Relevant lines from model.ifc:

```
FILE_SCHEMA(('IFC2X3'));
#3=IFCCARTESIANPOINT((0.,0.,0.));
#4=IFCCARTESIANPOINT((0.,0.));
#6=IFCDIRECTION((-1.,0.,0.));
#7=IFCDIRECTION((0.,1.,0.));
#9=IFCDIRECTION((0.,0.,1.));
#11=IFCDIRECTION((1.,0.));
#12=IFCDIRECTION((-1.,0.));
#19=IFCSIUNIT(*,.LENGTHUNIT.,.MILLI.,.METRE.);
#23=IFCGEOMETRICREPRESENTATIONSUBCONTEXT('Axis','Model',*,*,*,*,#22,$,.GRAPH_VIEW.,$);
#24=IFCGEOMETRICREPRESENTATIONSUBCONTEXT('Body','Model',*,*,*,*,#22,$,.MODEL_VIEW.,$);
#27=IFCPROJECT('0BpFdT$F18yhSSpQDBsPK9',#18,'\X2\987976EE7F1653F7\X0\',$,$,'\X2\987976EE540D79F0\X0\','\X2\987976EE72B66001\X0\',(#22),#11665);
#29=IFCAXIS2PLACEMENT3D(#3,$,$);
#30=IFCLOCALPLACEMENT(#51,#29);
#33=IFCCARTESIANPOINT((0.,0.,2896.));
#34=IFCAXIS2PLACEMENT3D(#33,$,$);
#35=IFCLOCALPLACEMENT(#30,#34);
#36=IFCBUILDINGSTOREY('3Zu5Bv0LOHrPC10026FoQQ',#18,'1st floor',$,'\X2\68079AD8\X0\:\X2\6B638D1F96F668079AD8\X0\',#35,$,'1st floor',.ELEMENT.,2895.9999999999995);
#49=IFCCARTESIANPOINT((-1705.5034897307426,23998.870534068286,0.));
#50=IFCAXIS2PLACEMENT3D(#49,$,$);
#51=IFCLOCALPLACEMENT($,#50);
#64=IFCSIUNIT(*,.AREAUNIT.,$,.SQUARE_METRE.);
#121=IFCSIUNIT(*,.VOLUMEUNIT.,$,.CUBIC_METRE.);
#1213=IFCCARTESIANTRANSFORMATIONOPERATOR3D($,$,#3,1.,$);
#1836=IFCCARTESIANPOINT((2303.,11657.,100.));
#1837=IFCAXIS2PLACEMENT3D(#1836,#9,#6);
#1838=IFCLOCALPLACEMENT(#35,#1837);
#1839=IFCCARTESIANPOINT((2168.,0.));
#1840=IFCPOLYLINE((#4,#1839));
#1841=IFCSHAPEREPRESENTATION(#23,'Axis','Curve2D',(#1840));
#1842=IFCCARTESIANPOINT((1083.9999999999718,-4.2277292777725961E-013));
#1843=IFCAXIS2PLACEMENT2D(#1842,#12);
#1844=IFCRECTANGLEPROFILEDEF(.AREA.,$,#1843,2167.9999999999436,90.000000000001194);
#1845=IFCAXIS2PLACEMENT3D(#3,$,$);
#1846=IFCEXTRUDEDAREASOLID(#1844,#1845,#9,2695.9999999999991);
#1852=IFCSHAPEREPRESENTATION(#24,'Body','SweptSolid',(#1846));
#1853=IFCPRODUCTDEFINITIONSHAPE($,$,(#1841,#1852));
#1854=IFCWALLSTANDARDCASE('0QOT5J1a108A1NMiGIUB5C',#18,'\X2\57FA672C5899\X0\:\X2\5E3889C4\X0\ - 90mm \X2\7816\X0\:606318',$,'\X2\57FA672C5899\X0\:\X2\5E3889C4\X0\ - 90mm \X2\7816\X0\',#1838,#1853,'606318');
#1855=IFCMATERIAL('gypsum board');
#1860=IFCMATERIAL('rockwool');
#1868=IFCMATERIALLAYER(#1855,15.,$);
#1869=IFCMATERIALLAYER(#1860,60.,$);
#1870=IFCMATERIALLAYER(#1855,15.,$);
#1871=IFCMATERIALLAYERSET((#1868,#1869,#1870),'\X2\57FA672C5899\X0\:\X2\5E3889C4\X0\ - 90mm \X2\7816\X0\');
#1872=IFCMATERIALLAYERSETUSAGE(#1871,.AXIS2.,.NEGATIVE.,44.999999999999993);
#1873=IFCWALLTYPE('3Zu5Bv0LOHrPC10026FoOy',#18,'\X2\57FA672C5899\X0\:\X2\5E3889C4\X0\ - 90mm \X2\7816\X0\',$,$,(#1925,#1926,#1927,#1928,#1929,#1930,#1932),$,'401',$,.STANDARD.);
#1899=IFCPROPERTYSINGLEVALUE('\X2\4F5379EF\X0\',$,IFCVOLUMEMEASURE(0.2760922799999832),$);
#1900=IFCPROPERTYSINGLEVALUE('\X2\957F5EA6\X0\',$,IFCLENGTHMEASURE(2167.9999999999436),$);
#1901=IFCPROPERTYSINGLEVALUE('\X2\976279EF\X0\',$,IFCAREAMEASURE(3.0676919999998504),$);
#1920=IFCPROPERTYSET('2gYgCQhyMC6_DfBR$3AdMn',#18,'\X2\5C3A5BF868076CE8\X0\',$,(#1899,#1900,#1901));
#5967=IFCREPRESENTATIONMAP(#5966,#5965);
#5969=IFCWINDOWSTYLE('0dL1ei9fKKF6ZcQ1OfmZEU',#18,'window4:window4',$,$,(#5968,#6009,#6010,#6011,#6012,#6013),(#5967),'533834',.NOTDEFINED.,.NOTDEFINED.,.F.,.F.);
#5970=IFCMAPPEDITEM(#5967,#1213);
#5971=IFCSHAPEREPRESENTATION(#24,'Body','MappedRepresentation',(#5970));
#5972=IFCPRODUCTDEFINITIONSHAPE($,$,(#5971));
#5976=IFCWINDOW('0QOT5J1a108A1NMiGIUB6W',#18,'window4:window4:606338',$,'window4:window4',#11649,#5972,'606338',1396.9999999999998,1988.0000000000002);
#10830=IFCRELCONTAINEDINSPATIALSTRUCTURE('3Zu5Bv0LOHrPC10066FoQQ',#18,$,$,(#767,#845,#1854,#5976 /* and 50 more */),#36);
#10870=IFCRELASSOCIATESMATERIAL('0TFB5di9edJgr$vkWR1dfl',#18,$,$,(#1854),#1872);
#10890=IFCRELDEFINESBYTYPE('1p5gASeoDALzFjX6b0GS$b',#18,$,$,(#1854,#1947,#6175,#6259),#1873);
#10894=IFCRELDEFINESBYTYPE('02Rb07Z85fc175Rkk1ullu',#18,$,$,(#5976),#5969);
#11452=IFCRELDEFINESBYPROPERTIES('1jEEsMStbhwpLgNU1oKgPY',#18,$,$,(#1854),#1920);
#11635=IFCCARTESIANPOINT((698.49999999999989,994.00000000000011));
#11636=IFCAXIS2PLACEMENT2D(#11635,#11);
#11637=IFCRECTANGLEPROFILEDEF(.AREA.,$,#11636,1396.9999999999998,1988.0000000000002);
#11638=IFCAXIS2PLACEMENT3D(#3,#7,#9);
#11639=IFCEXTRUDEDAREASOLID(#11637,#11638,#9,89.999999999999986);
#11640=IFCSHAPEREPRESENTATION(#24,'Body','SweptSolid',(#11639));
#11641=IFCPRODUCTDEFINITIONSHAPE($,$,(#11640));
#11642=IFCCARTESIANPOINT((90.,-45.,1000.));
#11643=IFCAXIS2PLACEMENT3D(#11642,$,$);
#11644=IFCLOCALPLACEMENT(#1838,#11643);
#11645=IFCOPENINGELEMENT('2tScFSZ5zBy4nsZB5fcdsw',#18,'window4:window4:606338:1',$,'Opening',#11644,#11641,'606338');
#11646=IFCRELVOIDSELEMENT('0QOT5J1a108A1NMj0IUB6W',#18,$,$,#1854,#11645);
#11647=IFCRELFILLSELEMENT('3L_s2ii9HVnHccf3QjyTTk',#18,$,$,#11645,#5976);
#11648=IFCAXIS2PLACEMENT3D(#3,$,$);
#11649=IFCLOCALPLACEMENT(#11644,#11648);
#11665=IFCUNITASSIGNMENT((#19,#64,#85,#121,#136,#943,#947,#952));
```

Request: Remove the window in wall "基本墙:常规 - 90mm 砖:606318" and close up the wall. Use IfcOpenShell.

```python
import ifcopenshell
import ifcopenshell.api.feature
import ifcopenshell.api.pset
import ifcopenshell.api.root
import ifcopenshell.geom
import ifcopenshell.util.element
import ifcopenshell.util.shape
import ifcopenshell.util.unit

model = ifcopenshell.open("model.ifc")
area_scale = ifcopenshell.util.unit.calculate_unit_scale(model, "AREAUNIT")
volume_scale = ifcopenshell.util.unit.calculate_unit_scale(model, "VOLUMEUNIT")
settings = ifcopenshell.geom.settings()


def volume(element):
    """Net volume in cubic metres, openings subtracted."""
    shape = ifcopenshell.geom.create_shape(settings, element)
    return ifcopenshell.util.shape.get_volume(shape.geometry)


window = model.by_guid("0QOT5J1a108A1NMiGIUB6W")
opening = window.FillsVoids[0].RelatingOpeningElement
wall = opening.VoidsElements[0].RelatingBuildingElement
before = volume(wall)

ifcopenshell.api.root.remove_product(model, product=window)
ifcopenshell.api.feature.remove_feature(model, feature=opening)

after = volume(wall)
thickness = 0.09  # wall thickness in metres

# Update the wall's stored quantities.
pset = model.by_id(ifcopenshell.util.element.get_pset(wall, "尺寸标注", should_inherit=False)["id"])
ifcopenshell.api.pset.edit_pset(model, pset=pset, properties={
    "体积": model.create_entity("IfcVolumeMeasure", after / volume_scale),
    "面积": model.create_entity("IfcAreaMeasure", after / thickness / area_scale),
})

print(f"wall volume {before:.3f} -> {after:.3f} m3")

model.write("model_rev.ifc")
```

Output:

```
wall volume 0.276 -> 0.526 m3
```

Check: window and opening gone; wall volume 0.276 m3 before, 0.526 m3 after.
